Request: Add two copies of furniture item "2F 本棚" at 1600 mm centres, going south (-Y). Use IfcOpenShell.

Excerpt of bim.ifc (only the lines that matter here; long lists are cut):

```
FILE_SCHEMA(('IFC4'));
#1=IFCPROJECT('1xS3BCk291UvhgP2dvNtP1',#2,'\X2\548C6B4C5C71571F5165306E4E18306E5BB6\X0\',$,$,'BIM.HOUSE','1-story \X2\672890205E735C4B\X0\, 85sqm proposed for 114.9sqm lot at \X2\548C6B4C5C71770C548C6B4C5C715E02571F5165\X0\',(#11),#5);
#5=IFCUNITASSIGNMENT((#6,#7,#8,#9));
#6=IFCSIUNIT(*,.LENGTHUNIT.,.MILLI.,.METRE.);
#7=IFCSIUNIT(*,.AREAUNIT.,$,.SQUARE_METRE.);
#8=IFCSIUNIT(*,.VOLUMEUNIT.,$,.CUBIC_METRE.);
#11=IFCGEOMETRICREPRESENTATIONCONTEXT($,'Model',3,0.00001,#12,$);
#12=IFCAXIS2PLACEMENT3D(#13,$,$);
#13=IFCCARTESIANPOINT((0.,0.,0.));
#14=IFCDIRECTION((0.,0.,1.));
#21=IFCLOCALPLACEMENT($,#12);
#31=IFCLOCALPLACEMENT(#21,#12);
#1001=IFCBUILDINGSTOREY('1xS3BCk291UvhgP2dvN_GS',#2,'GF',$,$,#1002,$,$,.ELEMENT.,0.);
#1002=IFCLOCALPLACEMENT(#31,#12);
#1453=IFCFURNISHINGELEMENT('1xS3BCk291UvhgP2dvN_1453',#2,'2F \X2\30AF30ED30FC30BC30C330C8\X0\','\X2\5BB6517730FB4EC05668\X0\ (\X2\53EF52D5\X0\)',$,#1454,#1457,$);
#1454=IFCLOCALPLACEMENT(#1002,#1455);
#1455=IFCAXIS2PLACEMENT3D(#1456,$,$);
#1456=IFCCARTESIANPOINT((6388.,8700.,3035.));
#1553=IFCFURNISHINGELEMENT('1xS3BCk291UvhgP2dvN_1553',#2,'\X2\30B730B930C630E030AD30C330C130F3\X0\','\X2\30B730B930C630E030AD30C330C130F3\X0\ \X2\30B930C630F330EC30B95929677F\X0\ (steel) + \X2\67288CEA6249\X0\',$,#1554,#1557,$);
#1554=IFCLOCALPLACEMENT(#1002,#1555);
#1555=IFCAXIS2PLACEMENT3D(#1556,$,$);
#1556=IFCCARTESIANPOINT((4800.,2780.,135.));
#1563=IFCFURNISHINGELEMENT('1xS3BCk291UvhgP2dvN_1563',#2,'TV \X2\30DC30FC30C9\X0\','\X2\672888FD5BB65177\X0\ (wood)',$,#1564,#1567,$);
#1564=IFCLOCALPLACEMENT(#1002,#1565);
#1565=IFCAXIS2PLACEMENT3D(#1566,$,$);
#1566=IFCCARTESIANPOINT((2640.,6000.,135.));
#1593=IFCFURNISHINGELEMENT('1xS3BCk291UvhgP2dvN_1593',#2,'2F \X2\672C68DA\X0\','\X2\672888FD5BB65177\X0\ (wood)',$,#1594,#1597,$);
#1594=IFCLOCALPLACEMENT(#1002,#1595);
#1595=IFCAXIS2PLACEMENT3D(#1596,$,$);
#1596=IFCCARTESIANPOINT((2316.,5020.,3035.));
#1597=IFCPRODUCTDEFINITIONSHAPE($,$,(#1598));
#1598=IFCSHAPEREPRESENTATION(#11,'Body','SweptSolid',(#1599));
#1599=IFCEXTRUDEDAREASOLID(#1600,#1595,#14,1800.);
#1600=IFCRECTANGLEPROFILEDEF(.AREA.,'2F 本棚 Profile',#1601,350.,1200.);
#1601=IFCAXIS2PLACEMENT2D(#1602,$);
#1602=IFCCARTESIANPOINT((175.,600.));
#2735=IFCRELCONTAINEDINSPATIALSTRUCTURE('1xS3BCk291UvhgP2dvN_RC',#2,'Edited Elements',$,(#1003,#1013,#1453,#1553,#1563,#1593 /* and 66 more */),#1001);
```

```python
import numpy as np
import ifcopenshell
import ifcopenshell.api.geometry
import ifcopenshell.api.root
import ifcopenshell.util.element
import ifcopenshell.util.placement

model = ifcopenshell.open("bim.ifc")


def reuse_history(source, copy):
    """copy_class also copies each property set's owner history, people and application; keep the originals."""
    for rel in copy.IsDefinedBy:
        if rel.is_a("IfcRelDefinesByProperties") and (history := rel.RelatingPropertyDefinition.OwnerHistory):
            rel.RelatingPropertyDefinition.OwnerHistory = source.OwnerHistory
            ifcopenshell.util.element.remove_deep2(model, history)


source = model.by_guid("1xS3BCk291UvhgP2dvN_1593")
base = ifcopenshell.util.placement.get_local_placement(source.ObjectPlacement)
step = np.array([0.0, -1.0, 0.0]) * 1600.0

for i in range(1, 3):
    copy = ifcopenshell.api.root.copy_class(model, product=source)
    copy.Representation = ifcopenshell.util.element.copy_deep(
        model, source.Representation, exclude=["IfcGeometricRepresentationContext", "IfcRepresentationMap"]
    )
    reuse_history(source, copy)
    matrix = base.copy()
    matrix[:3, 3] += i * step
    print("added at", matrix[:3, 3].round(3) + 0.0)
    ifcopenshell.api.geometry.edit_object_placement(model, product=copy, matrix=matrix, is_si=False)

model.write("bim-out.ifc")
```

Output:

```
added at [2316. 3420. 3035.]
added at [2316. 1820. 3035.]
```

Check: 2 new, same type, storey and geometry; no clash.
